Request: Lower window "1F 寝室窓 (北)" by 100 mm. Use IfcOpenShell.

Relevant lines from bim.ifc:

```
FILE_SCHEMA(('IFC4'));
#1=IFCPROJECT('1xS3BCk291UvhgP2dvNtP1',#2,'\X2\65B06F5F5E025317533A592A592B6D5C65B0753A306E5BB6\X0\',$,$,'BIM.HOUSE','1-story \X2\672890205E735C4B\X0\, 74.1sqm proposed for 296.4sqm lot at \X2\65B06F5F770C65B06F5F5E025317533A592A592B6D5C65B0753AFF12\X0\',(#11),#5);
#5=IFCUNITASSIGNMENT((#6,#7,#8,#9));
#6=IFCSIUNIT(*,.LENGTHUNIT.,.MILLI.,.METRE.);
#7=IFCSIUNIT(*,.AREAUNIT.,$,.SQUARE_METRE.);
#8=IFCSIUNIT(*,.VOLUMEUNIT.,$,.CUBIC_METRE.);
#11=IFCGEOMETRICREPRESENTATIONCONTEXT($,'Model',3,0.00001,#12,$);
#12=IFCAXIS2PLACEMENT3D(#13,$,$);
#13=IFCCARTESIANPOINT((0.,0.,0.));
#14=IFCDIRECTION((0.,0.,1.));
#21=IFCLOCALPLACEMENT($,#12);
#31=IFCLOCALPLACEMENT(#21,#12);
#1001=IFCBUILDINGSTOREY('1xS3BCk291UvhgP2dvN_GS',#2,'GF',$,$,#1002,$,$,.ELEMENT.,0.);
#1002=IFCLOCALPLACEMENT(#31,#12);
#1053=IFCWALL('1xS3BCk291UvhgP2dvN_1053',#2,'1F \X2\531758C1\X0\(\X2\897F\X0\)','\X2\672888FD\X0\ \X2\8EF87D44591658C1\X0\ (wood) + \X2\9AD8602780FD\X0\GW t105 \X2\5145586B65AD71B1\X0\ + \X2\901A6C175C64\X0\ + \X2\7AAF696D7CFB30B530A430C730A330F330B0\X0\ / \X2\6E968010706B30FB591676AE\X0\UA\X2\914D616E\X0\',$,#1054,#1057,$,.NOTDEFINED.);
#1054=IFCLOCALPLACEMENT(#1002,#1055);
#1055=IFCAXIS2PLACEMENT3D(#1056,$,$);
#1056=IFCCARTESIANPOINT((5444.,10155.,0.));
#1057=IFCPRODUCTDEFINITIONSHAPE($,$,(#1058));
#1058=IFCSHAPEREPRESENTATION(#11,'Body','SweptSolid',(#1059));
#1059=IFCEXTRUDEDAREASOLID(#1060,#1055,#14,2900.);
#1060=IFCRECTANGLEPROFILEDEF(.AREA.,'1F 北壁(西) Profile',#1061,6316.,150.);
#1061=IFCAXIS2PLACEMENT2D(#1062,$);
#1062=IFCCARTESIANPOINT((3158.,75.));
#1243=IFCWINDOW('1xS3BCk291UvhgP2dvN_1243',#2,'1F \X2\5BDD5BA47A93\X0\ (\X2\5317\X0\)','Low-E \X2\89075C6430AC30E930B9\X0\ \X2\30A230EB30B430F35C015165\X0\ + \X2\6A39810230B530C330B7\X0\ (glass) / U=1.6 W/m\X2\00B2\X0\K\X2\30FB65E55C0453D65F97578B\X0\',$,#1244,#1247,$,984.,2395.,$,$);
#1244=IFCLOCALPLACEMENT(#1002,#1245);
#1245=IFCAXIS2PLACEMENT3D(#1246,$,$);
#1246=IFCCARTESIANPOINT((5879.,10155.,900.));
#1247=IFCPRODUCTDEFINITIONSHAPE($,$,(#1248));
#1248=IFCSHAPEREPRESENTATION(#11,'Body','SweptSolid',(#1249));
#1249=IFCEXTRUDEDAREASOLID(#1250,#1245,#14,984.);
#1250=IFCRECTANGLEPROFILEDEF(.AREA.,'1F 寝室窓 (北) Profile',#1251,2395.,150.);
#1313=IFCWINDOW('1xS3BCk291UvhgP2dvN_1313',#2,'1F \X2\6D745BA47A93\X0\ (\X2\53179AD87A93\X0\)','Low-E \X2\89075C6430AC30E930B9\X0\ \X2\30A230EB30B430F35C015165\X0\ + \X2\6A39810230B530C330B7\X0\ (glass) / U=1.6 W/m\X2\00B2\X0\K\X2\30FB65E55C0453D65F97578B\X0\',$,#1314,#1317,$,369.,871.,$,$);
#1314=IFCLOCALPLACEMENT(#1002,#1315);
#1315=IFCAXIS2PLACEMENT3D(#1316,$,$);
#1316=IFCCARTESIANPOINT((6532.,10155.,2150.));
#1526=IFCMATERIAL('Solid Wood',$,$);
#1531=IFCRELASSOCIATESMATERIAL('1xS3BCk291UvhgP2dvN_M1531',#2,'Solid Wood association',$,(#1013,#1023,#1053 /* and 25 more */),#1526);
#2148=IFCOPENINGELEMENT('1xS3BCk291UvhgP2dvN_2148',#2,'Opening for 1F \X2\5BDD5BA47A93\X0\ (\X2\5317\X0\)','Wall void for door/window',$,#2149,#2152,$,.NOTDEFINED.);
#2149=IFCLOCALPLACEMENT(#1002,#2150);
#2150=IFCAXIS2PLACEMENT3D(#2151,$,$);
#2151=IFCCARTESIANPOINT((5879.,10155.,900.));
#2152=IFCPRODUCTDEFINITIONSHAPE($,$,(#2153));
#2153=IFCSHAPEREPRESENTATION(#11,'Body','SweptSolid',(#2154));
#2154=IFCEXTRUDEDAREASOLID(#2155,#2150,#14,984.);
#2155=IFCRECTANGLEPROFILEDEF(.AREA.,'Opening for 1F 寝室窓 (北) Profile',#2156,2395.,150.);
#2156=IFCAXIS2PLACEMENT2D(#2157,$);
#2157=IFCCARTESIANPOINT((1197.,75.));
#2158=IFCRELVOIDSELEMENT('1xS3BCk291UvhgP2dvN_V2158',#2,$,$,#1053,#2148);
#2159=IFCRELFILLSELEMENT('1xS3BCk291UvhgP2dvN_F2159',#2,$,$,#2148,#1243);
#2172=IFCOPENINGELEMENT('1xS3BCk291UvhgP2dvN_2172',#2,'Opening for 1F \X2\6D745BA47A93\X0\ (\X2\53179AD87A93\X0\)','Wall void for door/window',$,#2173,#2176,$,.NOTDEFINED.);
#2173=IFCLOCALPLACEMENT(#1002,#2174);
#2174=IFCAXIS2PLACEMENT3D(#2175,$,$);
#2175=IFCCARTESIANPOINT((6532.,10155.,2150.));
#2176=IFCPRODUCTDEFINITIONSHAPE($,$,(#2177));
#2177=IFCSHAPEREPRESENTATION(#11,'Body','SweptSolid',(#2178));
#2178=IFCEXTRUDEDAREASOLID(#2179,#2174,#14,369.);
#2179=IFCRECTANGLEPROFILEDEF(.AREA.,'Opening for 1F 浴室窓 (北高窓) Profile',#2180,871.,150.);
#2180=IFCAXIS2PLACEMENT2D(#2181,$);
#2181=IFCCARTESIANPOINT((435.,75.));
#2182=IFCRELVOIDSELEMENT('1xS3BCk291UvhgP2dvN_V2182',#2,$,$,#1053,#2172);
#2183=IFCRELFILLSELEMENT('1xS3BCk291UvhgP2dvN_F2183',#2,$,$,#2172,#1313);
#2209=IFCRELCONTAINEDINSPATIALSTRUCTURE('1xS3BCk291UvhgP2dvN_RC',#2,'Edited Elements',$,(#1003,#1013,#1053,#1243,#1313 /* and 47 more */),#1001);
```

```python
import numpy as np
import ifcopenshell
import ifcopenshell.api.geometry
import ifcopenshell.util.placement
import ifcopenshell.util.unit

model = ifcopenshell.open("bim.ifc")
unit_scale = ifcopenshell.util.unit.calculate_unit_scale(model)

window = model.by_guid("1xS3BCk291UvhgP2dvN_1243")
opening = window.FillsVoids[0].RelatingOpeningElement
dz = -100.0

shift = np.array([0.0, 0.0, dz])
# The window is not placed relative to its opening, so move both.
for product in (opening, window):
    matrix = ifcopenshell.util.placement.get_local_placement(product.ObjectPlacement)
    matrix[:3, 3] += shift
    ifcopenshell.api.geometry.edit_object_placement(model, product=product, matrix=matrix, is_si=False)

print(f"moved by {dz * unit_scale:+.3f} m")

model.write("bim-out.ifc")
```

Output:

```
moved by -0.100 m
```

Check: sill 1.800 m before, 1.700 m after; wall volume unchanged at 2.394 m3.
